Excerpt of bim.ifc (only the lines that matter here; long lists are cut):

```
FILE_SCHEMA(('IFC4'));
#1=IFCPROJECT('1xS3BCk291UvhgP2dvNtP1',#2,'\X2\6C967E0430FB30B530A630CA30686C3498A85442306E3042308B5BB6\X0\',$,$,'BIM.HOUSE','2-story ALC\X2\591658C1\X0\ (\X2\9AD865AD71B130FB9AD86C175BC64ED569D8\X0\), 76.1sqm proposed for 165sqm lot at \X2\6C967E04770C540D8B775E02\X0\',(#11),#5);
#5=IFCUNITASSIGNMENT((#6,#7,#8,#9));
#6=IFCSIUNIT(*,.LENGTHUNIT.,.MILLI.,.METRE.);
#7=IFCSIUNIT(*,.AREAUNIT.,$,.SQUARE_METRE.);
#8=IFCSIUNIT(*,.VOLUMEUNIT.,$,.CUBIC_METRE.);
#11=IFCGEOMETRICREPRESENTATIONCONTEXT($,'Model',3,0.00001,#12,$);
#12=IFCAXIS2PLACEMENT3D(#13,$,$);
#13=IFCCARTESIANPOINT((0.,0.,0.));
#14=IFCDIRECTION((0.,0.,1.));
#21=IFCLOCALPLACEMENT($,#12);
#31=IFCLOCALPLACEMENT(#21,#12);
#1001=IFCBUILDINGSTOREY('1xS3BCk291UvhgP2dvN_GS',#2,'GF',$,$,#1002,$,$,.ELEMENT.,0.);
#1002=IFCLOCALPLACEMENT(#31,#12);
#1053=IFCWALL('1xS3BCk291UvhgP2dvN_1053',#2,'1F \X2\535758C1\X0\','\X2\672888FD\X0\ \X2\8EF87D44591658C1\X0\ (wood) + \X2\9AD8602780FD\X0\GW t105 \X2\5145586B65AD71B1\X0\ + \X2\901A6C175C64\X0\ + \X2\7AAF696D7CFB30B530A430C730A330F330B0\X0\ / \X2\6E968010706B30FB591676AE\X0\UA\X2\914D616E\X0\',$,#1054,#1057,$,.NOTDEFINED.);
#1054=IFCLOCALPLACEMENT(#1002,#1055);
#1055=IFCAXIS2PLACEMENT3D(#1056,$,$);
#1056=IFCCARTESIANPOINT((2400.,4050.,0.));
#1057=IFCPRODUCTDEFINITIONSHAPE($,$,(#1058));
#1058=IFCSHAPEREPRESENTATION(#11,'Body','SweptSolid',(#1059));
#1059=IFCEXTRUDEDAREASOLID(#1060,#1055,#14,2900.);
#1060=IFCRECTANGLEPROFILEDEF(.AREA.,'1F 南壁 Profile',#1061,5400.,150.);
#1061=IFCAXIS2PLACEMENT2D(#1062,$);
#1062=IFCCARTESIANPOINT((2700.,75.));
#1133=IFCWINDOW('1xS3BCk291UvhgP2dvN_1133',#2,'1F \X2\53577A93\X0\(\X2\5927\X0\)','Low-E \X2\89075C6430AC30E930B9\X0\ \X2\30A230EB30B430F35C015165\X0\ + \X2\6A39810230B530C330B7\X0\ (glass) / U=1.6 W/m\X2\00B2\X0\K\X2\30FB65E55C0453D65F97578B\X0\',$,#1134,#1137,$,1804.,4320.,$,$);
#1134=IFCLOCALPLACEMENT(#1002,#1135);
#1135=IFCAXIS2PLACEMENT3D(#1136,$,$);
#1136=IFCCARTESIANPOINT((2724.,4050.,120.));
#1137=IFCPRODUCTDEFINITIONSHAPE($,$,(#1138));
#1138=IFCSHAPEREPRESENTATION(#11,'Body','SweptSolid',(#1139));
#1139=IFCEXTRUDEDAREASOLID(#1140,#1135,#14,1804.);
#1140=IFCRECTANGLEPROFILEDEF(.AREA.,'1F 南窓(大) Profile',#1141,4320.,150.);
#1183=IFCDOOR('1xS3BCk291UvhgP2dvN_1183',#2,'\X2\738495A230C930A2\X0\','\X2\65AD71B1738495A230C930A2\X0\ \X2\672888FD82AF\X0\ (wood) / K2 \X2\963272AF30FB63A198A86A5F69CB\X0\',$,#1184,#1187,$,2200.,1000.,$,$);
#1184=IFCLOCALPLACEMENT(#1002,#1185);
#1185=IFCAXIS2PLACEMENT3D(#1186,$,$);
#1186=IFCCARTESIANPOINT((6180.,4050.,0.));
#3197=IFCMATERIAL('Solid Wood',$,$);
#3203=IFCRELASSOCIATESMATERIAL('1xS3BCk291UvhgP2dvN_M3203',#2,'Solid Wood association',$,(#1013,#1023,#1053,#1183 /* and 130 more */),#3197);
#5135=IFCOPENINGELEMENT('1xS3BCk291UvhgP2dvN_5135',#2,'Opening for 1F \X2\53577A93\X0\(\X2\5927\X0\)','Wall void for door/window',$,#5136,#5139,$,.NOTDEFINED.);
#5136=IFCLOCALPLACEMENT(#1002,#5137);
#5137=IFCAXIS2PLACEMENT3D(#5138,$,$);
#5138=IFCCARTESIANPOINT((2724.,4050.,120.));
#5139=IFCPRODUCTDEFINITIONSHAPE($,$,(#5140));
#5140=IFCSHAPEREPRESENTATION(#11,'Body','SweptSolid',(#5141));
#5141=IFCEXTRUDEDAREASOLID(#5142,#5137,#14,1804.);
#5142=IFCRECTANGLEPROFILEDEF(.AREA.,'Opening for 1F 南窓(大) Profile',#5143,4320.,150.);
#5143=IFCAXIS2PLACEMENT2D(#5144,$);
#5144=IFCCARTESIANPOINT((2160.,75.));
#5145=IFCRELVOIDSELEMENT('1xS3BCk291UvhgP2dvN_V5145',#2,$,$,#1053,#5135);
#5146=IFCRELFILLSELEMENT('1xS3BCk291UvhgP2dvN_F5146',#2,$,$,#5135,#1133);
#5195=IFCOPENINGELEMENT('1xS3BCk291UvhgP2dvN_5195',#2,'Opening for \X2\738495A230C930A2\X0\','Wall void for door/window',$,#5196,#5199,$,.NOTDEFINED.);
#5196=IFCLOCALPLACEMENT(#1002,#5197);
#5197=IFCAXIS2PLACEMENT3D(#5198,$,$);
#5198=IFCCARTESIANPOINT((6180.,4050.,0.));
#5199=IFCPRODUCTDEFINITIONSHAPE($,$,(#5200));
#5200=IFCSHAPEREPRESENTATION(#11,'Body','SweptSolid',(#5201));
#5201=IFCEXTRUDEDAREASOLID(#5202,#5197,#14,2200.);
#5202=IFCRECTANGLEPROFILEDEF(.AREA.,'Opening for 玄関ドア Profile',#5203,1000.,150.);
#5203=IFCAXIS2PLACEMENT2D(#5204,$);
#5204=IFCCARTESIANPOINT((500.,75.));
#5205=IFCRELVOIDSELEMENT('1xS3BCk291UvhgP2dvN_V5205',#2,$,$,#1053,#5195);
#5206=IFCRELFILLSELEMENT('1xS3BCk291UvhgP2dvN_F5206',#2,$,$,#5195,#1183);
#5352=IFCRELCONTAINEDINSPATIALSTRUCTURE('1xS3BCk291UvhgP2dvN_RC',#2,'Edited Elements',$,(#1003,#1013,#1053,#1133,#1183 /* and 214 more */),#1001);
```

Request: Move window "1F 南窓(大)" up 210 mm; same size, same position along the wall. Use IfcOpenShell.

```python
import numpy as np
import ifcopenshell
import ifcopenshell.api.geometry
import ifcopenshell.util.placement
import ifcopenshell.util.unit

model = ifcopenshell.open("bim.ifc")
unit_scale = ifcopenshell.util.unit.calculate_unit_scale(model)

window = model.by_id(1133)
opening = window.FillsVoids[0].RelatingOpeningElement
dz = 0.21 / unit_scale

shift = np.array([0.0, 0.0, dz])
# The window is not placed relative to its opening, so move both.
for product in (opening, window):
    matrix = ifcopenshell.util.placement.get_local_placement(product.ObjectPlacement)
    matrix[:3, 3] += shift
    ifcopenshell.api.geometry.edit_object_placement(model, product=product, matrix=matrix, is_si=False)

print(f"moved by {dz * unit_scale:+.3f} m")

model.write("bim_edited.ifc")
```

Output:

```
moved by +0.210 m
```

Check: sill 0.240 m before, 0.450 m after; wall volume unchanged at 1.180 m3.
